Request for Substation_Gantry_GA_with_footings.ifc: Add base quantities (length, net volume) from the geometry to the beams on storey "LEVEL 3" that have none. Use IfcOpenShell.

First a look at what the model holds.

```python
import ifcopenshell
import ifcopenshell.util.element
import ifcopenshell.util.unit

model = ifcopenshell.open("Substation_Gantry_GA_with_footings.ifc")
print(model.schema)
for unit_type in ("LENGTHUNIT", "AREAUNIT", "VOLUMEUNIT"):
    print(unit_type, ifcopenshell.util.unit.calculate_unit_scale(model, unit_type))
storey = next(s for s in model.by_type("IfcBuildingStorey") if s.Name == "LEVEL 3")
beams = [e for e in ifcopenshell.util.element.get_decomposition(storey) if e.is_a("IfcBeam")]
for e in sorted(beams, key=lambda e: e.id()):
    print(e.id(), e.is_a(), e.Name, list(ifcopenshell.util.element.get_psets(e, qtos_only=True)), sep=" | ")
```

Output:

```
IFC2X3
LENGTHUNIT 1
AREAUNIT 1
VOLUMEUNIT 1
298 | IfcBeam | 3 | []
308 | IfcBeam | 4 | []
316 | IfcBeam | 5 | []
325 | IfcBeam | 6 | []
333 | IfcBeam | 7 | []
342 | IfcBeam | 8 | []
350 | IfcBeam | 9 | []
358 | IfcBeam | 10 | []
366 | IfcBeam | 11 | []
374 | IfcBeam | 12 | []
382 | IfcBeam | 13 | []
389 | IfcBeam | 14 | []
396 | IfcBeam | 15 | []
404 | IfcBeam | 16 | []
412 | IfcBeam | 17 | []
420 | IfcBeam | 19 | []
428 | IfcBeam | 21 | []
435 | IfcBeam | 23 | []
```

```python
import ifcopenshell
import ifcopenshell.api.pset
import ifcopenshell.geom
import ifcopenshell.util.element
import ifcopenshell.util.shape
import ifcopenshell.util.unit

model = ifcopenshell.open("Substation_Gantry_GA_with_footings.ifc")
unit_scale = ifcopenshell.util.unit.calculate_unit_scale(model)
volume_scale = ifcopenshell.util.unit.calculate_unit_scale(model, "VOLUMEUNIT")
settings = ifcopenshell.geom.settings()

storey = next(s for s in model.by_type("IfcBuildingStorey") if s.Name == "LEVEL 3")
beams = [e for e in ifcopenshell.util.element.get_decomposition(storey) if e.is_a("IfcBeam")]

for e in sorted(beams, key=lambda e: e.id()):
    if ifcopenshell.util.element.get_psets(e, qtos_only=True, should_inherit=False):
        continue
    # Geometry comes back in metres, in the element's own axes.
    shape = ifcopenshell.geom.create_shape(settings, e)
    values = {
        "Length": ifcopenshell.util.shape.get_max_xyz(shape.geometry) / unit_scale,
        "NetVolume": ifcopenshell.util.shape.get_volume(shape.geometry) / volume_scale,
    }
    qto = ifcopenshell.api.pset.add_qto(model, product=e, name="BaseQuantities")
    ifcopenshell.api.pset.edit_qto(model, qto=qto, properties=values)
    print(e.id(), {k: round(v, 3) for k, v in values.items()})

model.write("Substation_Gantry_GA_with_footings_edited.ifc")
```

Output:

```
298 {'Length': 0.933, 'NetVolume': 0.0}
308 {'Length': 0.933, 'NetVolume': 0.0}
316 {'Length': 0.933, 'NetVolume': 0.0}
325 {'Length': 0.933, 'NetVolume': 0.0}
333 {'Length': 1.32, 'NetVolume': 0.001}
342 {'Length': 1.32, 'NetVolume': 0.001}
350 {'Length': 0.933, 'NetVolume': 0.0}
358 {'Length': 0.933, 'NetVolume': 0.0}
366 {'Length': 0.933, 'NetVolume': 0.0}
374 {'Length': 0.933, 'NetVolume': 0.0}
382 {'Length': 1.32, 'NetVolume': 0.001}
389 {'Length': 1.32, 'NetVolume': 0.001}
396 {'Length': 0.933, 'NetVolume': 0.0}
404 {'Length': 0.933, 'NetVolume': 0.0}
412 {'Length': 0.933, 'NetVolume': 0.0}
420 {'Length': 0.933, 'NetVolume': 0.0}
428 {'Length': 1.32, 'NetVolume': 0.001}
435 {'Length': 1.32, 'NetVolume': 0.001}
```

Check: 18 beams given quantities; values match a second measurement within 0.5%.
